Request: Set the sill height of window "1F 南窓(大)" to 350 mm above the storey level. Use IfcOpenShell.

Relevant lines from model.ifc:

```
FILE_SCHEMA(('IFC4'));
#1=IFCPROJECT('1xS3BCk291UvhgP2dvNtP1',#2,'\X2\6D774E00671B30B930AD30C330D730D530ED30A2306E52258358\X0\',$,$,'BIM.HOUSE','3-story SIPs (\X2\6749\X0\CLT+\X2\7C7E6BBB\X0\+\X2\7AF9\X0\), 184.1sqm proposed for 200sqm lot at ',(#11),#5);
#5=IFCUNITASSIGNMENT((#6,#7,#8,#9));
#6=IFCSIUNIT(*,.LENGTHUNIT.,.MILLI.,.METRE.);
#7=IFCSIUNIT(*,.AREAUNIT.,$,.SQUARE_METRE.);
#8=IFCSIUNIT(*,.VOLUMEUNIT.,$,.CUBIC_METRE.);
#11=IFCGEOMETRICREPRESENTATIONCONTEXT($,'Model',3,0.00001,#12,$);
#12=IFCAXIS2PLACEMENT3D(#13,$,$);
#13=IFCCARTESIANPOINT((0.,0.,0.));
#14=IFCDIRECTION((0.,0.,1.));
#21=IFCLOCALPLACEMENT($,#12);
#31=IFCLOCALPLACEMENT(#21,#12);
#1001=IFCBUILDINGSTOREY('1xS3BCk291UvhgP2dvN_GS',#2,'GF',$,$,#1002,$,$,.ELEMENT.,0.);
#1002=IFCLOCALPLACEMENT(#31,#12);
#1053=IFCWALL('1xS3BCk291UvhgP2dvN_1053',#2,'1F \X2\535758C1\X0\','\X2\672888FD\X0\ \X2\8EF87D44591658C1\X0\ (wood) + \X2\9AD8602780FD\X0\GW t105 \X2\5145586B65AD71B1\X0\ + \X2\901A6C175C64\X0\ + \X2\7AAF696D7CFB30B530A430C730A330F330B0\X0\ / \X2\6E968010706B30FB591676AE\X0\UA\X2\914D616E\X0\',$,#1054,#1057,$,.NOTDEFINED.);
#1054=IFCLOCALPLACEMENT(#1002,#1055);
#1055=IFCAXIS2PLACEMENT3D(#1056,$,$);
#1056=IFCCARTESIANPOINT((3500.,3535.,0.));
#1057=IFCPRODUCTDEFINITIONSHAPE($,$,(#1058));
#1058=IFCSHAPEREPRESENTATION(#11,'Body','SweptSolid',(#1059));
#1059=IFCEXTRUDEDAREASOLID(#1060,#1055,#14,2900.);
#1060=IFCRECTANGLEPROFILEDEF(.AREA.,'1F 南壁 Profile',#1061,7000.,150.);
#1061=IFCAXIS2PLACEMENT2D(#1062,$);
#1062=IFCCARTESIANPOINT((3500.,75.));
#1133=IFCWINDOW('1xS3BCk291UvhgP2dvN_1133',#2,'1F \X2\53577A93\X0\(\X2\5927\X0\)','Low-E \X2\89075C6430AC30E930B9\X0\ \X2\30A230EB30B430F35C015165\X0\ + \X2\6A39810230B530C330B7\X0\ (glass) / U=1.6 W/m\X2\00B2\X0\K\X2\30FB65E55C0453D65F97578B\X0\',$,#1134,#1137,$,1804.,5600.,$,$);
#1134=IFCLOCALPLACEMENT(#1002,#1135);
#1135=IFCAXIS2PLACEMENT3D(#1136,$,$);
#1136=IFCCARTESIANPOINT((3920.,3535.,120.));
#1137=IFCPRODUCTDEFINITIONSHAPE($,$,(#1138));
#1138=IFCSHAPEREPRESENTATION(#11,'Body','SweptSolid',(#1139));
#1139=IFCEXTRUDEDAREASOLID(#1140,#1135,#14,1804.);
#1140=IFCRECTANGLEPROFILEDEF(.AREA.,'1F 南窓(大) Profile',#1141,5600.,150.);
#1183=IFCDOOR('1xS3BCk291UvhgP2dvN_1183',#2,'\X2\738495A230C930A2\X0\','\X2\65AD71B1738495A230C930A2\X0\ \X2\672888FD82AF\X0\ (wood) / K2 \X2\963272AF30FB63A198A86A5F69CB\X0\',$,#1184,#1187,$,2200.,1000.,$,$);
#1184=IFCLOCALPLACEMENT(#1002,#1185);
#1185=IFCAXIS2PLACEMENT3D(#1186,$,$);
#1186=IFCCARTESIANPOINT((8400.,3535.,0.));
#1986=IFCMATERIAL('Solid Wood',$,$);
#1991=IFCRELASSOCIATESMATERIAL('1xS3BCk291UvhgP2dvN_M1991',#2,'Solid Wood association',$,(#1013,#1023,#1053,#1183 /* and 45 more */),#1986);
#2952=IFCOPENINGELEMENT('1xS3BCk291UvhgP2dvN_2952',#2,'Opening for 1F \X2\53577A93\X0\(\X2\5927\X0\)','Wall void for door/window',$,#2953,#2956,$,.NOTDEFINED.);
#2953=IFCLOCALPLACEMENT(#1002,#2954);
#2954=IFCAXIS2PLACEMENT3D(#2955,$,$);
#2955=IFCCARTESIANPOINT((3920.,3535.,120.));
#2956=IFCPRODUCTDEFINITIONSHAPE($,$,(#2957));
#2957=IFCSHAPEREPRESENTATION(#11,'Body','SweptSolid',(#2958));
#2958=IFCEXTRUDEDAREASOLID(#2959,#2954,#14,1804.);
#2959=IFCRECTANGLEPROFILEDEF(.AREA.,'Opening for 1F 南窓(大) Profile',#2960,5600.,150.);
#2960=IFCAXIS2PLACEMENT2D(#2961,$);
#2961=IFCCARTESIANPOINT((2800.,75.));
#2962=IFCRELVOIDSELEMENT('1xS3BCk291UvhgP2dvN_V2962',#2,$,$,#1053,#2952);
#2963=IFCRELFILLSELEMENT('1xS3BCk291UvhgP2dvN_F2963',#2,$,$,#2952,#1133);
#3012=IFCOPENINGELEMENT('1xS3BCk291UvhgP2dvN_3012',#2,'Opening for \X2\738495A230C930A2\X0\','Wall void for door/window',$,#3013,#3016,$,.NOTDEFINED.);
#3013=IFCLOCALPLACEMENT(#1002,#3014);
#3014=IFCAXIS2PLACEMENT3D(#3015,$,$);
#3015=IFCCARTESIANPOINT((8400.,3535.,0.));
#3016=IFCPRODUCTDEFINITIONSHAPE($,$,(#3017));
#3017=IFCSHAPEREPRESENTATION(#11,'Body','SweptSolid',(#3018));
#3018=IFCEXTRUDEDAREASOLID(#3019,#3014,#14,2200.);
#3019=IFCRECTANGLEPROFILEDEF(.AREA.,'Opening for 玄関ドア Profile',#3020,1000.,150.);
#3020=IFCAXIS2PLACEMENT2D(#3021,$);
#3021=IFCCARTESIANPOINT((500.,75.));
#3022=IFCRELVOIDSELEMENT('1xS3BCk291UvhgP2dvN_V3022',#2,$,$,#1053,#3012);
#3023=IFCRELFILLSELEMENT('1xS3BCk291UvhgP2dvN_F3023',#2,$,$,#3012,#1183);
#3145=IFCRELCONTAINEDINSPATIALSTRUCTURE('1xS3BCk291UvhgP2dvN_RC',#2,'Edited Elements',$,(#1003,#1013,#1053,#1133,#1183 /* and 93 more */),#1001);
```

```python
import numpy as np
import ifcopenshell
import ifcopenshell.api.geometry
import ifcopenshell.geom
import ifcopenshell.util.element
import ifcopenshell.util.placement
import ifcopenshell.util.shape
import ifcopenshell.util.unit

model = ifcopenshell.open("model.ifc")
unit_scale = ifcopenshell.util.unit.calculate_unit_scale(model)

window = model.by_id(1133)
opening = window.FillsVoids[0].RelatingOpeningElement
storey = ifcopenshell.util.element.get_container(window, ifc_class="IfcBuildingStorey")
level = ifcopenshell.util.placement.get_local_placement(storey.ObjectPlacement)[2, 3]

# The opening's origin need not be at the sill, so measure its lowest point.
shape = ifcopenshell.geom.create_shape(ifcopenshell.geom.settings(), opening)
bottom = ifcopenshell.util.shape.get_shape_bottom_elevation(shape, shape.geometry) / unit_scale
dz = level + 350.0 - bottom

shift = np.array([0.0, 0.0, dz])
# The window is not placed relative to its opening, so move both.
for product in (opening, window):
    matrix = ifcopenshell.util.placement.get_local_placement(product.ObjectPlacement)
    matrix[:3, 3] += shift
    ifcopenshell.api.geometry.edit_object_placement(model, product=product, matrix=matrix, is_si=False)

print(f"moved by {dz * unit_scale:+.3f} m")

model.write("model_edited.ifc")
```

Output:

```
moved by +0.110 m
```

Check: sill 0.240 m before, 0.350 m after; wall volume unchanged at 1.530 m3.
